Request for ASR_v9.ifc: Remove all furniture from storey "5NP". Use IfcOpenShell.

First a look at what the model holds.

```python
import ifcopenshell
import ifcopenshell.util.element

model = ifcopenshell.open("ASR_v9.ifc")
print(model.schema)
storey = next(s for s in model.by_type("IfcBuildingStorey") if s.Name == "5NP")
furniture = [e for e in ifcopenshell.util.element.get_decomposition(storey) if e.is_a("IfcFurnishingElement")]
seen = {}
for e in furniture:
    element_type = ifcopenshell.util.element.get_type(e)
    name = element_type.Name if element_type not in (None, e) else None
    seen[name] = seen.get(name, 0) + 1
for name, count in sorted(seen.items(), key=str):
    print(count, "x", name)
```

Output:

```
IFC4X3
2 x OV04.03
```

```python
import ifcopenshell
import ifcopenshell.api.root
import ifcopenshell.util.element

model = ifcopenshell.open("ASR_v9.ifc")

storey = next(s for s in model.by_type("IfcBuildingStorey") if s.Name == "5NP")
furniture = [e for e in ifcopenshell.util.element.get_decomposition(storey) if e.is_a("IfcFurnishingElement")]

for e in furniture:
    ifcopenshell.api.root.remove_product(model, product=e)
print(len(furniture), "removed")

model.write("ASR_v9_rev.ifc")
```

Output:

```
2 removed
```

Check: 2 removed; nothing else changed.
